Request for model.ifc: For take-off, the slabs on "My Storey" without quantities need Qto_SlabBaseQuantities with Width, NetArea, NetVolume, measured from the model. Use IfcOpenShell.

First a look at what the model holds.

```python
import ifcopenshell
import ifcopenshell.util.element
import ifcopenshell.util.unit

model = ifcopenshell.open("model.ifc")
print(model.schema)
for unit_type in ("LENGTHUNIT", "AREAUNIT", "VOLUMEUNIT"):
    print(unit_type, ifcopenshell.util.unit.calculate_unit_scale(model, unit_type))
storey = next(s for s in model.by_type("IfcBuildingStorey") if s.Name == "My Storey")
slabs = [e for e in ifcopenshell.util.element.get_decomposition(storey) if e.is_a("IfcSlab")]
for e in sorted(slabs, key=lambda e: e.id()):
    print(e.id(), e.is_a(), e.Name, list(ifcopenshell.util.element.get_psets(e, qtos_only=True)), sep=" | ")
```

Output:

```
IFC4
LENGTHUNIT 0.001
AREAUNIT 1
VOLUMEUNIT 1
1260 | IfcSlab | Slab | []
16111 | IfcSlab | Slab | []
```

```python
import ifcopenshell
import ifcopenshell.api.pset
import ifcopenshell.geom
import ifcopenshell.util.element
import ifcopenshell.util.shape
import ifcopenshell.util.unit

model = ifcopenshell.open("model.ifc")
unit_scale = ifcopenshell.util.unit.calculate_unit_scale(model)
area_scale = ifcopenshell.util.unit.calculate_unit_scale(model, "AREAUNIT")
volume_scale = ifcopenshell.util.unit.calculate_unit_scale(model, "VOLUMEUNIT")
settings = ifcopenshell.geom.settings()

storey = next(s for s in model.by_type("IfcBuildingStorey") if s.Name == "My Storey")
slabs = [e for e in ifcopenshell.util.element.get_decomposition(storey) if e.is_a("IfcSlab")]

for e in sorted(slabs, key=lambda e: e.id()):
    if ifcopenshell.util.element.get_psets(e, qtos_only=True, should_inherit=False):
        continue
    # Geometry comes back in metres, in the element's own axes.
    shape = ifcopenshell.geom.create_shape(settings, e)
    values = {
        "Width": ifcopenshell.util.shape.get_z(shape.geometry) / unit_scale,
        "NetArea": ifcopenshell.util.shape.get_footprint_area(shape.geometry) / area_scale,
        "NetVolume": ifcopenshell.util.shape.get_volume(shape.geometry) / volume_scale,
    }
    qto = ifcopenshell.api.pset.add_qto(model, product=e, name="Qto_SlabBaseQuantities")
    ifcopenshell.api.pset.edit_qto(model, qto=qto, properties=values)
    print(e.id(), {k: round(v, 3) for k, v in values.items()})

model.write("model_rev.ifc")
```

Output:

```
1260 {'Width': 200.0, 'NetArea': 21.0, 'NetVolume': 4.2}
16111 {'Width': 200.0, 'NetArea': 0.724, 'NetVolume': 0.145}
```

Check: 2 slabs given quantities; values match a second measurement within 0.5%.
